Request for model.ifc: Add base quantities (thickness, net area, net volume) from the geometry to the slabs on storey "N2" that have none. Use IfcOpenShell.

First a look at what the model holds.

```python
import ifcopenshell
import ifcopenshell.util.element
import ifcopenshell.util.unit

model = ifcopenshell.open("model.ifc")
print(model.schema)
for unit_type in ("LENGTHUNIT", "AREAUNIT", "VOLUMEUNIT"):
    print(unit_type, ifcopenshell.util.unit.calculate_unit_scale(model, unit_type))
storey = next(s for s in model.by_type("IfcBuildingStorey") if s.Name == "N2")
slabs = [e for e in ifcopenshell.util.element.get_decomposition(storey) if e.is_a("IfcSlab")]
for e in sorted(slabs, key=lambda e: e.id()):
    print(e.id(), e.is_a(), e.Name, list(ifcopenshell.util.element.get_psets(e, qtos_only=True)), sep=" | ")
```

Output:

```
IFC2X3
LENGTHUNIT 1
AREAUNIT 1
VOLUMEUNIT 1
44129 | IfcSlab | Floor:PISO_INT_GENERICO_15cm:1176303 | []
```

```python
import ifcopenshell
import ifcopenshell.api.pset
import ifcopenshell.geom
import ifcopenshell.util.element
import ifcopenshell.util.shape
import ifcopenshell.util.unit

model = ifcopenshell.open("model.ifc")
unit_scale = ifcopenshell.util.unit.calculate_unit_scale(model)
area_scale = ifcopenshell.util.unit.calculate_unit_scale(model, "AREAUNIT")
volume_scale = ifcopenshell.util.unit.calculate_unit_scale(model, "VOLUMEUNIT")
settings = ifcopenshell.geom.settings()

storey = next(s for s in model.by_type("IfcBuildingStorey") if s.Name == "N2")
slabs = [e for e in ifcopenshell.util.element.get_decomposition(storey) if e.is_a("IfcSlab")]

for e in sorted(slabs, key=lambda e: e.id()):
    if ifcopenshell.util.element.get_psets(e, qtos_only=True, should_inherit=False):
        continue
    # Geometry comes back in metres, in the element's own axes.
    shape = ifcopenshell.geom.create_shape(settings, e)
    values = {
        "Width": ifcopenshell.util.shape.get_z(shape.geometry) / unit_scale,
        "NetArea": ifcopenshell.util.shape.get_footprint_area(shape.geometry) / area_scale,
        "NetVolume": ifcopenshell.util.shape.get_volume(shape.geometry) / volume_scale,
    }
    qto = ifcopenshell.api.pset.add_qto(model, product=e, name="BaseQuantities")
    ifcopenshell.api.pset.edit_qto(model, qto=qto, properties=values)
    print(e.id(), {k: round(v, 3) for k, v in values.items()})

model.write("model_edited.ifc")
```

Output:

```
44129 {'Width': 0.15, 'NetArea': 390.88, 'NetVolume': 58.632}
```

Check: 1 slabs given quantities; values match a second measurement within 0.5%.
